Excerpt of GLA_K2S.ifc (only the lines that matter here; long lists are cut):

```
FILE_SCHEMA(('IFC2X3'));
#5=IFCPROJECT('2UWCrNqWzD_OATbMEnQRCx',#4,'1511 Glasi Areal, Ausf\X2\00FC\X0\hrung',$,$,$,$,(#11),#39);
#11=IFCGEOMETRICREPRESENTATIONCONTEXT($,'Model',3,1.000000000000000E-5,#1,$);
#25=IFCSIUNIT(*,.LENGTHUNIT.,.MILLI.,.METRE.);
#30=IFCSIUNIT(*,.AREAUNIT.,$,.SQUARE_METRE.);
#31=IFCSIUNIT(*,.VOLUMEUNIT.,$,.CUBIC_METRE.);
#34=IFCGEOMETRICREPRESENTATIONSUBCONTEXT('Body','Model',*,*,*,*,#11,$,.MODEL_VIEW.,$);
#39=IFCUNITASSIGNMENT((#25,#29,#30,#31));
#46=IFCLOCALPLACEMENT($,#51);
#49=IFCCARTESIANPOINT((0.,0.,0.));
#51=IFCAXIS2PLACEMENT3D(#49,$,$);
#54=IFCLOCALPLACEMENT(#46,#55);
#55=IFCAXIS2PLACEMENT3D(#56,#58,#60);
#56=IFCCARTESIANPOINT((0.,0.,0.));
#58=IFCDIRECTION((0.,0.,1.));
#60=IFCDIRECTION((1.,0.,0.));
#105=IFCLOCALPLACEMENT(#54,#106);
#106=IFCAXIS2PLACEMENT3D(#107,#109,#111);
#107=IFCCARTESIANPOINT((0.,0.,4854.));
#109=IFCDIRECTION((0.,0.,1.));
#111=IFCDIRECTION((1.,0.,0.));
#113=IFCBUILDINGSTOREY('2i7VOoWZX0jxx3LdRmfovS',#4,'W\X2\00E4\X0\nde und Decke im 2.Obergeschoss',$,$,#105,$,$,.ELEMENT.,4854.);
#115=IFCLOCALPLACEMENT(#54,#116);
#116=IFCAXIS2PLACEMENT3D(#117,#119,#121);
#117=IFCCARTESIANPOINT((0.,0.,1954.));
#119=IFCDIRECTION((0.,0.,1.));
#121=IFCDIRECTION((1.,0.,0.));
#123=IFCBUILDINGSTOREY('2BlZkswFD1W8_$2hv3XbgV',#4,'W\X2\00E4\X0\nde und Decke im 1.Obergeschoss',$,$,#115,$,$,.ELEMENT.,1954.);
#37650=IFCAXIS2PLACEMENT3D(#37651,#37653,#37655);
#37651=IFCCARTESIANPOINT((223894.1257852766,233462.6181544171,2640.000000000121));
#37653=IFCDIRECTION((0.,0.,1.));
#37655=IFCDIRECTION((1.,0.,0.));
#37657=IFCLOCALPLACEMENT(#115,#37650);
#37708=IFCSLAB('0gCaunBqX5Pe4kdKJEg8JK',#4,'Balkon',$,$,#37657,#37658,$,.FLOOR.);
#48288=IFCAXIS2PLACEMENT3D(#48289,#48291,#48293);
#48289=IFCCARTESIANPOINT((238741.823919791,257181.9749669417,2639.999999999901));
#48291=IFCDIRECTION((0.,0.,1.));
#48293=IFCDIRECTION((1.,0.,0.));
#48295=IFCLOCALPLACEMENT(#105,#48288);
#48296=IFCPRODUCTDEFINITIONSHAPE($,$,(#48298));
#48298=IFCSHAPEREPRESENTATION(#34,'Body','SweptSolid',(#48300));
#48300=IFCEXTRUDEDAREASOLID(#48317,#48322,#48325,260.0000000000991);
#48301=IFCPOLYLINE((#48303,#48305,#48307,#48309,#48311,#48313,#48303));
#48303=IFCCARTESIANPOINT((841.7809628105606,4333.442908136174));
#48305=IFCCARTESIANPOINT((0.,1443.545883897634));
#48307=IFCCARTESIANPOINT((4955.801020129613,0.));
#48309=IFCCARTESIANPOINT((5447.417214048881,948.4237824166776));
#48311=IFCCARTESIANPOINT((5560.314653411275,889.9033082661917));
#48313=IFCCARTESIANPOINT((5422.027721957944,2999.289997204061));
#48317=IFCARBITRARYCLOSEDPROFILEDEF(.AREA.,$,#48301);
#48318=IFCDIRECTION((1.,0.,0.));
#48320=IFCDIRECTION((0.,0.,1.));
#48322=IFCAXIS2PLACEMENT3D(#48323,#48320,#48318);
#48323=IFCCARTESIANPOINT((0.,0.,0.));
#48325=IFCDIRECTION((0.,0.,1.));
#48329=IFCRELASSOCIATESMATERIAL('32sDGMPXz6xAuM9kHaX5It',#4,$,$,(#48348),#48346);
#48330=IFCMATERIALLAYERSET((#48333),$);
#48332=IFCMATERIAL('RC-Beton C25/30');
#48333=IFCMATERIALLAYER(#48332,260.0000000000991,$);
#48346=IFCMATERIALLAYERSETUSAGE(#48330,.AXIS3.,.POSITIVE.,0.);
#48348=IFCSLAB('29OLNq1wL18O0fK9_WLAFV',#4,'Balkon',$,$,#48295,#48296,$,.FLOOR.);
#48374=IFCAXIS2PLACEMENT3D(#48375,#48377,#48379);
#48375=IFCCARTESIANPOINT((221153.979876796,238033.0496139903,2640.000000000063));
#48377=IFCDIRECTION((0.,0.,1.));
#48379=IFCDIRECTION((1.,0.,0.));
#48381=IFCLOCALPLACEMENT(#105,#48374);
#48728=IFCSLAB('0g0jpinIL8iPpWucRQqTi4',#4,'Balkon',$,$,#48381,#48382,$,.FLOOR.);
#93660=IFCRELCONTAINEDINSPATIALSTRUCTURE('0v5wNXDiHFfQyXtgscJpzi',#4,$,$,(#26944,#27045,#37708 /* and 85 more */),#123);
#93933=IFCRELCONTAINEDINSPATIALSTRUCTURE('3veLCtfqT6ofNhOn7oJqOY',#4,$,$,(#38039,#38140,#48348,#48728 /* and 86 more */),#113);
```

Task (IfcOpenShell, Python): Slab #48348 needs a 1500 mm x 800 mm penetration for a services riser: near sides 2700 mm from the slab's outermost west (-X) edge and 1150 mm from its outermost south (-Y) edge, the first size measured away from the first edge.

```python
import numpy as np
import ifcopenshell
import ifcopenshell.api.feature
import ifcopenshell.api.geometry
import ifcopenshell.api.root
import ifcopenshell.geom
import ifcopenshell.util.placement
import ifcopenshell.util.representation
import ifcopenshell.util.shape
import ifcopenshell.util.unit

model = ifcopenshell.open("GLA_K2S.ifc")
unit_scale = ifcopenshell.util.unit.calculate_unit_scale(model)
settings = ifcopenshell.geom.settings()


def volume(element):
    """Net volume in cubic metres, openings subtracted."""
    shape = ifcopenshell.geom.create_shape(settings, element)
    return ifcopenshell.util.shape.get_volume(shape.geometry)


slab = model.by_guid("29OLNq1wL18O0fK9_WLAFV")
before = volume(slab)

# Extent in the slab's own axes, in metres. The edges named are its -X and -Y sides.
slab_shape = ifcopenshell.geom.create_shape(settings, slab)
vertices = ifcopenshell.util.shape.get_vertices(slab_shape.geometry)
x_min, y_min, bottom = vertices.min(axis=0)
top = vertices[:, 2].max()

opening = ifcopenshell.api.root.create_entity(model, ifc_class="IfcOpeningElement", name="Services riser opening")
context = ifcopenshell.util.representation.get_context(model, "Model", "Body", "MODEL_VIEW")
width, depth = 1.5, 0.8
outline = [(0.0, 0.0), (width, 0.0), (width, depth), (0.0, depth), (0.0, 0.0)]
# Overshoot both faces by 50 mm so the cut is clean.
shape = ifcopenshell.api.geometry.add_slab_representation(
    model, context=context, depth=top - bottom + 0.1, polyline=outline
)
ifcopenshell.api.geometry.assign_representation(model, product=opening, representation=shape)

matrix = ifcopenshell.util.placement.get_local_placement(slab.ObjectPlacement)
matrix[:, 3] = matrix @ np.append(np.array([x_min + 2.7, y_min + 1.15, bottom - 0.05]) / unit_scale, 1.0)
ifcopenshell.api.geometry.edit_object_placement(model, product=opening, matrix=matrix, is_si=False)
ifcopenshell.api.feature.add_feature(model, feature=opening, element=slab)

after = volume(slab)

print(f"slab volume {before:.3f} -> {after:.3f} m3")

model.write("GLA_K2S_updated.ifc")
```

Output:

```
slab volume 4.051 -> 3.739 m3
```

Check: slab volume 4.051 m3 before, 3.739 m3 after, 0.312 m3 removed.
